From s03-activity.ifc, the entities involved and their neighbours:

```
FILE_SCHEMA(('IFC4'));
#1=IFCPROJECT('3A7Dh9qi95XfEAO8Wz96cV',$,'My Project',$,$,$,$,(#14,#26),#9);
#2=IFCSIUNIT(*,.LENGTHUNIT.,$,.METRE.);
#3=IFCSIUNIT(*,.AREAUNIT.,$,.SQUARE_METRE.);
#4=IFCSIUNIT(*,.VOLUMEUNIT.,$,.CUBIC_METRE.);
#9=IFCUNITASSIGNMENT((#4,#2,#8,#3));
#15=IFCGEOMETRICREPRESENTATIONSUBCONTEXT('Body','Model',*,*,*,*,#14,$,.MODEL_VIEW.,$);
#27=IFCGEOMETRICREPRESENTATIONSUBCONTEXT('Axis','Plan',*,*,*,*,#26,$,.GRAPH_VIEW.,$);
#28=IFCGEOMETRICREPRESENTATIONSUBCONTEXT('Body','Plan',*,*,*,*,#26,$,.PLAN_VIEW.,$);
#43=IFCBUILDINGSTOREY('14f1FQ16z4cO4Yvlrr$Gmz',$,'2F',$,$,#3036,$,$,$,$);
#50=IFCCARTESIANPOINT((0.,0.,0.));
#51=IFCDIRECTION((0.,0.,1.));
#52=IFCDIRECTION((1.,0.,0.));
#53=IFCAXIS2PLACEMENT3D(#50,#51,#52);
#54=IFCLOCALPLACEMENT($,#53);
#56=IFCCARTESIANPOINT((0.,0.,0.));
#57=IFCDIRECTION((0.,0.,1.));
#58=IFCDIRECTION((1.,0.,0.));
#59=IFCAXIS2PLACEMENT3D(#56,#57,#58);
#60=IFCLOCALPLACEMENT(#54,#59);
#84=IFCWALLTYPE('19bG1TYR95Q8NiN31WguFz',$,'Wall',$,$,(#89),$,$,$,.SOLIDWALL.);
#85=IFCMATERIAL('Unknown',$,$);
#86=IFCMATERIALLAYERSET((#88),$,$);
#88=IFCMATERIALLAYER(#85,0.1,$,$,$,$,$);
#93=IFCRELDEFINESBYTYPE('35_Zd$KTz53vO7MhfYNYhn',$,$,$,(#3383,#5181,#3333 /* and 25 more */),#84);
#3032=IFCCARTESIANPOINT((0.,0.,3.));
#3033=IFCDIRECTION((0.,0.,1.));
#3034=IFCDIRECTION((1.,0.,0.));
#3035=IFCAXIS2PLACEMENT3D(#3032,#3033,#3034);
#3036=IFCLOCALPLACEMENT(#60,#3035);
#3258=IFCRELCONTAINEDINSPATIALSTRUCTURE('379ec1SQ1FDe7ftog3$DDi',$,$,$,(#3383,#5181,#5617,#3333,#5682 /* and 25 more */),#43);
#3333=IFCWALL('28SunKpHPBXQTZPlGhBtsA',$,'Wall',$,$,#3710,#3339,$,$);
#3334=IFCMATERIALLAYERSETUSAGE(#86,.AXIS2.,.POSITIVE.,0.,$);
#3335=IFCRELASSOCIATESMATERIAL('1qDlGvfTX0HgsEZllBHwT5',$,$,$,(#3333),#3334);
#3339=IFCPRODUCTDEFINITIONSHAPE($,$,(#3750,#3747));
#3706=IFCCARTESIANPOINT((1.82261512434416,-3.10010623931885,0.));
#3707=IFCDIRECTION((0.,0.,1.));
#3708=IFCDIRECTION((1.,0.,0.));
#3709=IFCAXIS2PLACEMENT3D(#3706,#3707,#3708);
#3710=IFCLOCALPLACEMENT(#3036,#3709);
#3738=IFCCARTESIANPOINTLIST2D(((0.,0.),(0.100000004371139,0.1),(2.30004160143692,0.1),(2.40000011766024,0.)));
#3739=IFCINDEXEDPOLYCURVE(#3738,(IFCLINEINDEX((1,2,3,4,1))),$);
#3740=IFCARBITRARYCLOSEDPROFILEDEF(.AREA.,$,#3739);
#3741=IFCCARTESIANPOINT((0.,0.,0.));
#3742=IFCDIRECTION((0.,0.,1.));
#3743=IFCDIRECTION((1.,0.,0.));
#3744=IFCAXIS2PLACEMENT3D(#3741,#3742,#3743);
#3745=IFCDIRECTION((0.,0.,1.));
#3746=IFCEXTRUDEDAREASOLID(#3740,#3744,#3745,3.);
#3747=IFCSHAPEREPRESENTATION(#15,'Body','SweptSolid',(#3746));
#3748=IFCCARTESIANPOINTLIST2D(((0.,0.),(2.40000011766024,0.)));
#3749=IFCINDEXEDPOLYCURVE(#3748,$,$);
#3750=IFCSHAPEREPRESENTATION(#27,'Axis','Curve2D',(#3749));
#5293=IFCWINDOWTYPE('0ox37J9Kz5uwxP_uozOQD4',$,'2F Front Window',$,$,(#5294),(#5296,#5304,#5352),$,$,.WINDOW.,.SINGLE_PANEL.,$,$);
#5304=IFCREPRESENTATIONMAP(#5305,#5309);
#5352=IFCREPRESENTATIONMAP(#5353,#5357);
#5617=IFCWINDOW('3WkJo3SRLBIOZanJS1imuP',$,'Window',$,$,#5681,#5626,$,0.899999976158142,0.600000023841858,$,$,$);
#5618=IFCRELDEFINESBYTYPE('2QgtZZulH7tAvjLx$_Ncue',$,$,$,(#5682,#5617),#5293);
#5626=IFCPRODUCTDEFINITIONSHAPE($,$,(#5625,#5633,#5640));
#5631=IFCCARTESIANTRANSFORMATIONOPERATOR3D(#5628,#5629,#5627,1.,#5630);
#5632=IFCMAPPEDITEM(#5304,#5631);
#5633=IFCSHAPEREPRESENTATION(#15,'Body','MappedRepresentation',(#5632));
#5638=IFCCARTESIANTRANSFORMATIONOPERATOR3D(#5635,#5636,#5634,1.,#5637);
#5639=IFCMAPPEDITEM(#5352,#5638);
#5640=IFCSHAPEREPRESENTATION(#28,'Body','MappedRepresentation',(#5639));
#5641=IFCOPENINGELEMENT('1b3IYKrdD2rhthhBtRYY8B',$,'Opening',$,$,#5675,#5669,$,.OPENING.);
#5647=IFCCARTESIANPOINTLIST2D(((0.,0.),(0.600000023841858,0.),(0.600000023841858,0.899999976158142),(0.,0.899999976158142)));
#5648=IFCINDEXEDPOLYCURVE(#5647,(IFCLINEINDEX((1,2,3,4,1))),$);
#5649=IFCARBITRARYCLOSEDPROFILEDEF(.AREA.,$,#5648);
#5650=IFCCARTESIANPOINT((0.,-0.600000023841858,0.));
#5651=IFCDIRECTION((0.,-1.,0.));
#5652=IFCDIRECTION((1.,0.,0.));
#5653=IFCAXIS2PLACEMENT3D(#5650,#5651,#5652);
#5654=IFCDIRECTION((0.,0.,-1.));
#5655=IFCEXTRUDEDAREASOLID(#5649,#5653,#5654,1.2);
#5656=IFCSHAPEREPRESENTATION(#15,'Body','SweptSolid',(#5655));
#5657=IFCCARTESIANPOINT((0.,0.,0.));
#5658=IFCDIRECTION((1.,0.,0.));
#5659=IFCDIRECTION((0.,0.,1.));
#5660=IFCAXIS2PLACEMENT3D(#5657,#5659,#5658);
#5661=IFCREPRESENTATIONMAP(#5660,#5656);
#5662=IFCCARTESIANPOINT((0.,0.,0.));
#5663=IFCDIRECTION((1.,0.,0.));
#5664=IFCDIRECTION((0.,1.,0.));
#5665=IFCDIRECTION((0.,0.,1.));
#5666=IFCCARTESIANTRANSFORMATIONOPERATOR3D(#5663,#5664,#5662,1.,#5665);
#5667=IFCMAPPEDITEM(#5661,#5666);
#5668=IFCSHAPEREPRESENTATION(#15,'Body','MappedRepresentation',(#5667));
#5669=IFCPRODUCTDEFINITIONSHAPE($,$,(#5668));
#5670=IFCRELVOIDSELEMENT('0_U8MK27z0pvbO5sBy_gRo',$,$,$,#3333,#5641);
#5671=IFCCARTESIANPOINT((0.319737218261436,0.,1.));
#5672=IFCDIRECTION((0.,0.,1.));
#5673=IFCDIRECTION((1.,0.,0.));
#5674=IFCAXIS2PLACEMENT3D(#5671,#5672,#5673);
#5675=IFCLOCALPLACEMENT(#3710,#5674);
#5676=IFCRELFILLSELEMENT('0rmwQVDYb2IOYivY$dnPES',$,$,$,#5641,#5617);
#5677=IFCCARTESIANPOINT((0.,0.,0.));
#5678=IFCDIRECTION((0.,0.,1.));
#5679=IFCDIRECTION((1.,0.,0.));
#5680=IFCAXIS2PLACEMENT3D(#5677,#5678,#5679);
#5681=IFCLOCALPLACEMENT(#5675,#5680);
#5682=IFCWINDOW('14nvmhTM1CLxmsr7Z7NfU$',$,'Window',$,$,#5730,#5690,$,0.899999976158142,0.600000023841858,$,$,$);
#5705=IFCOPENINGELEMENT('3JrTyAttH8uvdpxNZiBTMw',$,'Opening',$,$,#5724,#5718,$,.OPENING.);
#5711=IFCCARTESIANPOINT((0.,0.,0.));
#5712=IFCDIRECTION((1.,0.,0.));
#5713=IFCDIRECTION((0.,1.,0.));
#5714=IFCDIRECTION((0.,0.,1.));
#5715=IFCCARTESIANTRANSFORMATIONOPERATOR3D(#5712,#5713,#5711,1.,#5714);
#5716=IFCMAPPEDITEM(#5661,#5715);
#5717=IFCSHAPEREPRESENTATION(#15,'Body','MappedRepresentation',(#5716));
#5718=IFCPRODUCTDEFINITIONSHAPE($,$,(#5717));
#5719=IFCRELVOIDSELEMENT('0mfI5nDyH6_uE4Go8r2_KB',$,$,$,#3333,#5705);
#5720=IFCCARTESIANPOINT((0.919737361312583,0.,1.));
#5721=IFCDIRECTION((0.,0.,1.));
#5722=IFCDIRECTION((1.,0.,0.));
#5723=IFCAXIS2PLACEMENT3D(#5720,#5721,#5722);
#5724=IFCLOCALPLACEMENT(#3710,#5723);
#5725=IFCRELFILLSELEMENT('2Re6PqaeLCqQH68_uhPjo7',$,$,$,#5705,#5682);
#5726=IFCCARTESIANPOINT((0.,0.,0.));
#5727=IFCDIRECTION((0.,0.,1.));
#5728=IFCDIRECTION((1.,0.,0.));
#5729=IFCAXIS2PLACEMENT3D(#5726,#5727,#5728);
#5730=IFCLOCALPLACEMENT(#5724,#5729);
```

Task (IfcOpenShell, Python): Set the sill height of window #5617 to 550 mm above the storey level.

```python
import numpy as np
import ifcopenshell
import ifcopenshell.api.geometry
import ifcopenshell.geom
import ifcopenshell.util.element
import ifcopenshell.util.placement
import ifcopenshell.util.shape
import ifcopenshell.util.unit

model = ifcopenshell.open("s03-activity.ifc")
unit_scale = ifcopenshell.util.unit.calculate_unit_scale(model)

window = model.by_id(5617)
opening = window.FillsVoids[0].RelatingOpeningElement
storey = ifcopenshell.util.element.get_container(window, ifc_class="IfcBuildingStorey")
level = ifcopenshell.util.placement.get_local_placement(storey.ObjectPlacement)[2, 3]

# The opening's origin need not be at the sill, so measure its lowest point.
shape = ifcopenshell.geom.create_shape(ifcopenshell.geom.settings(), opening)
bottom = ifcopenshell.util.shape.get_shape_bottom_elevation(shape, shape.geometry) / unit_scale
dz = level + 0.55 - bottom

shift = np.array([0.0, 0.0, dz])
# The window is placed relative to its opening, so it follows when the opening moves.
matrix = ifcopenshell.util.placement.get_local_placement(opening.ObjectPlacement)
matrix[:3, 3] += shift
ifcopenshell.api.geometry.edit_object_placement(
    model, product=opening, matrix=matrix, is_si=False, should_transform_children=True
)

print(f"moved by {dz * unit_scale:+.3f} m")

model.write("s03-activity_v2.ifc")
```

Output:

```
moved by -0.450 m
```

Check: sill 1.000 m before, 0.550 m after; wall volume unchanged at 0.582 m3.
